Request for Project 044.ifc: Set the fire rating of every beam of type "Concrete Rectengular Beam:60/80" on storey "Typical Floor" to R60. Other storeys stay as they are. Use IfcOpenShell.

First a look at what the model holds.

```python
import ifcopenshell
import ifcopenshell.util.element

model = ifcopenshell.open("Project 044.ifc")
print(model.schema)
storey = next(s for s in model.by_type("IfcBuildingStorey") if s.Name == "Typical Floor")
beams = [e for e in ifcopenshell.util.element.get_decomposition(storey) if e.is_a("IfcBeam")]
seen = {}
for e in beams:
    element_type = ifcopenshell.util.element.get_type(e)
    key = (element_type.Name if element_type != e and element_type else None, ifcopenshell.util.element.get_pset(e, "Pset_BeamCommon", "FireRating"))
    seen[key] = seen.get(key, 0) + 1
for (name, value), count in sorted(seen.items(), key=str):
    print(count, "x", name, "|", value)
```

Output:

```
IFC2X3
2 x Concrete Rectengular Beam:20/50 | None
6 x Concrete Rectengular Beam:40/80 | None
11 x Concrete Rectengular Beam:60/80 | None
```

```python
import ifcopenshell
import ifcopenshell.api.pset
import ifcopenshell.util.element

model = ifcopenshell.open("Project 044.ifc")

storey = next(s for s in model.by_type("IfcBuildingStorey") if s.Name == "Typical Floor")
beams = [e for e in ifcopenshell.util.element.get_decomposition(storey) if e.is_a("IfcBeam")]

count = 0
for e in beams:
    element_type = ifcopenshell.util.element.get_type(e)
    if element_type in (None, e) or element_type.Name != "Concrete Rectengular Beam:60/80":
        continue
    # add_pset returns the element's existing set when there is one.
    pset = ifcopenshell.api.pset.add_pset(model, product=e, name="Pset_BeamCommon")
    ifcopenshell.api.pset.edit_pset(model, pset=pset, properties={"FireRating": "R60"})
    count += 1

print(count, "beams updated")

model.write("Project 044_updated.ifc")
```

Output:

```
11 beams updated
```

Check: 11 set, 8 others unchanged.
